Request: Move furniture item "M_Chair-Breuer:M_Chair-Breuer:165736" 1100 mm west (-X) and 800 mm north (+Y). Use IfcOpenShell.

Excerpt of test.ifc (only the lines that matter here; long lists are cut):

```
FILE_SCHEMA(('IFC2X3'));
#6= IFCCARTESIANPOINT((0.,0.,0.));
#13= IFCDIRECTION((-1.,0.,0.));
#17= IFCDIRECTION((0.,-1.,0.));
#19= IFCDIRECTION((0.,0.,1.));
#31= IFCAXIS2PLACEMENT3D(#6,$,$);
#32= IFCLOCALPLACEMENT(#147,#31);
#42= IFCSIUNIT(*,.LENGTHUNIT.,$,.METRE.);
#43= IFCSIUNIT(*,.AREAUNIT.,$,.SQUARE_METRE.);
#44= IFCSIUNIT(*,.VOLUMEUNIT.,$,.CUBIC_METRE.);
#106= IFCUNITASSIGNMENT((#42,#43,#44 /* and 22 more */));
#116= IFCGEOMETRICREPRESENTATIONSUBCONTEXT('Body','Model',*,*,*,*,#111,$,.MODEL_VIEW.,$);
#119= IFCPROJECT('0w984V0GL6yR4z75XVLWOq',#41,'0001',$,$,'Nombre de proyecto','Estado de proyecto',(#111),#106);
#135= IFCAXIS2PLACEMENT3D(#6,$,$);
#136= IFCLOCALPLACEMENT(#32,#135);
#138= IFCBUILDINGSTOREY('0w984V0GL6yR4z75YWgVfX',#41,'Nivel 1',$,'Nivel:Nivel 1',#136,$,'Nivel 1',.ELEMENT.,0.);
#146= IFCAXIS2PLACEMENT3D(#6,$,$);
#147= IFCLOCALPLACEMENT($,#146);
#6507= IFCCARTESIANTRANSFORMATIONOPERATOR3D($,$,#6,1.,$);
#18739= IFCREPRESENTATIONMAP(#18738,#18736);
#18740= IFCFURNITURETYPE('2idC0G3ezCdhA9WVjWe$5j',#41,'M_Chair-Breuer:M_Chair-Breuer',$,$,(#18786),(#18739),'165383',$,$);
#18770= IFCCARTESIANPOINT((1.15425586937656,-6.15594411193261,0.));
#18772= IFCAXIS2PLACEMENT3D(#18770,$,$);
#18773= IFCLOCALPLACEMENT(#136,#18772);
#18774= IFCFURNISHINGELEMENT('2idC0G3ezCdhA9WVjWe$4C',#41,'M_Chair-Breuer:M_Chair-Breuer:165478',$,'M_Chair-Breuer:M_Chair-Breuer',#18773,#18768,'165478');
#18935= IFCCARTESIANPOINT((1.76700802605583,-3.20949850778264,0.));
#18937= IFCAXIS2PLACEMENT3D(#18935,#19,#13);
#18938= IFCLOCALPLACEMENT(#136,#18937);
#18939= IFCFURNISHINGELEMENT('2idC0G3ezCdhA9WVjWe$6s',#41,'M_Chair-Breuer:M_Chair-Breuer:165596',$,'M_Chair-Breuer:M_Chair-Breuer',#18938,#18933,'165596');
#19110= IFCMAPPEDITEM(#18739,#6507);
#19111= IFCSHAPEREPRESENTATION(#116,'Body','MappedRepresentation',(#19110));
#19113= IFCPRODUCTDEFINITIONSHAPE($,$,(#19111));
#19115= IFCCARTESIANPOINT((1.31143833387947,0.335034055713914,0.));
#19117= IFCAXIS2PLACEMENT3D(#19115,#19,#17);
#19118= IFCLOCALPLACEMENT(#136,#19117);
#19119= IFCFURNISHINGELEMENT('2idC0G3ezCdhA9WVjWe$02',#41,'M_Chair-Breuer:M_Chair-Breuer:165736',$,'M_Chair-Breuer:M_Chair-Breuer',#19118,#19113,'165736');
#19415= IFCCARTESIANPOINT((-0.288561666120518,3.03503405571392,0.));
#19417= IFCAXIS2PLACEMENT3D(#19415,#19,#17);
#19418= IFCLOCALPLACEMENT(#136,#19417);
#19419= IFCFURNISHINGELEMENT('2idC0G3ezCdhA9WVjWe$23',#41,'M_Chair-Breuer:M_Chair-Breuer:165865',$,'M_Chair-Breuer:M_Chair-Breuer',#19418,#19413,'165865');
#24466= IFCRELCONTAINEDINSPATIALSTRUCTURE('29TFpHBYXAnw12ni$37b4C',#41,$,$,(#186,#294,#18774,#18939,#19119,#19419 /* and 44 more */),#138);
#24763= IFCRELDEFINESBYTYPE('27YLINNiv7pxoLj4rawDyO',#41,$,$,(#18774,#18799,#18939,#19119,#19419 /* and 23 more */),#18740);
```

```python
import ifcopenshell
import ifcopenshell.api.geometry
import ifcopenshell.util.placement
import ifcopenshell.util.unit

model = ifcopenshell.open("test.ifc")
unit_scale = ifcopenshell.util.unit.calculate_unit_scale(model)

item = model.by_guid("2idC0G3ezCdhA9WVjWe$02")
matrix = ifcopenshell.util.placement.get_local_placement(item.ObjectPlacement)
matrix[0, 3] -= 1.1 / unit_scale
matrix[1, 3] += 0.8 / unit_scale
ifcopenshell.api.geometry.edit_object_placement(model, product=item, matrix=matrix, is_si=False)

print(ifcopenshell.util.placement.get_local_placement(item.ObjectPlacement).round(3) + 0.0)

model.write("test_edited.ifc")
```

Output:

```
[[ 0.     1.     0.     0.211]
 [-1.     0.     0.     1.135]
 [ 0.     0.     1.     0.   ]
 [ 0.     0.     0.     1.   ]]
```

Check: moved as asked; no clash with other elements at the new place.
